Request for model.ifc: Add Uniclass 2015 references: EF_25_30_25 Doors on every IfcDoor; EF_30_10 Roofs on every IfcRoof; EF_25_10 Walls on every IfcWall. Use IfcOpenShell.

First a look at what the model holds.

```python
import ifcopenshell

model = ifcopenshell.open("model.ifc")
print(model.schema)
print("classifications:", [c.Name for c in model.by_type("IfcClassification")])
for ifc_class in ("IfcDoor", "IfcRoof", "IfcStair", "IfcWall", "IfcWindow"):
    print(ifc_class, len(model.by_type(ifc_class)))
```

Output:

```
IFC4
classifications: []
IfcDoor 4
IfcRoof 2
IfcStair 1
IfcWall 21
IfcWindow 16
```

```python
import ifcopenshell
import ifcopenshell.api.classification

model = ifcopenshell.open("model.ifc")

system = ifcopenshell.api.classification.add_classification(model, classification="Uniclass 2015")

codes = {
    "IfcDoor": ("EF_25_30_25", "Doors"),
    "IfcRoof": ("EF_30_10", "Roofs"),
    "IfcWall": ("EF_25_10", "Walls"),
}
for ifc_class, (code, name) in codes.items():
    products = model.by_type(ifc_class)
    ifcopenshell.api.classification.add_reference(
        model, products=products, classification=system, identification=code, name=name
    )
    print(code, len(products))

model.write("model_v2.ifc")
```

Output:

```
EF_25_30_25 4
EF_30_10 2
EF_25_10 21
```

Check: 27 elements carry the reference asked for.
